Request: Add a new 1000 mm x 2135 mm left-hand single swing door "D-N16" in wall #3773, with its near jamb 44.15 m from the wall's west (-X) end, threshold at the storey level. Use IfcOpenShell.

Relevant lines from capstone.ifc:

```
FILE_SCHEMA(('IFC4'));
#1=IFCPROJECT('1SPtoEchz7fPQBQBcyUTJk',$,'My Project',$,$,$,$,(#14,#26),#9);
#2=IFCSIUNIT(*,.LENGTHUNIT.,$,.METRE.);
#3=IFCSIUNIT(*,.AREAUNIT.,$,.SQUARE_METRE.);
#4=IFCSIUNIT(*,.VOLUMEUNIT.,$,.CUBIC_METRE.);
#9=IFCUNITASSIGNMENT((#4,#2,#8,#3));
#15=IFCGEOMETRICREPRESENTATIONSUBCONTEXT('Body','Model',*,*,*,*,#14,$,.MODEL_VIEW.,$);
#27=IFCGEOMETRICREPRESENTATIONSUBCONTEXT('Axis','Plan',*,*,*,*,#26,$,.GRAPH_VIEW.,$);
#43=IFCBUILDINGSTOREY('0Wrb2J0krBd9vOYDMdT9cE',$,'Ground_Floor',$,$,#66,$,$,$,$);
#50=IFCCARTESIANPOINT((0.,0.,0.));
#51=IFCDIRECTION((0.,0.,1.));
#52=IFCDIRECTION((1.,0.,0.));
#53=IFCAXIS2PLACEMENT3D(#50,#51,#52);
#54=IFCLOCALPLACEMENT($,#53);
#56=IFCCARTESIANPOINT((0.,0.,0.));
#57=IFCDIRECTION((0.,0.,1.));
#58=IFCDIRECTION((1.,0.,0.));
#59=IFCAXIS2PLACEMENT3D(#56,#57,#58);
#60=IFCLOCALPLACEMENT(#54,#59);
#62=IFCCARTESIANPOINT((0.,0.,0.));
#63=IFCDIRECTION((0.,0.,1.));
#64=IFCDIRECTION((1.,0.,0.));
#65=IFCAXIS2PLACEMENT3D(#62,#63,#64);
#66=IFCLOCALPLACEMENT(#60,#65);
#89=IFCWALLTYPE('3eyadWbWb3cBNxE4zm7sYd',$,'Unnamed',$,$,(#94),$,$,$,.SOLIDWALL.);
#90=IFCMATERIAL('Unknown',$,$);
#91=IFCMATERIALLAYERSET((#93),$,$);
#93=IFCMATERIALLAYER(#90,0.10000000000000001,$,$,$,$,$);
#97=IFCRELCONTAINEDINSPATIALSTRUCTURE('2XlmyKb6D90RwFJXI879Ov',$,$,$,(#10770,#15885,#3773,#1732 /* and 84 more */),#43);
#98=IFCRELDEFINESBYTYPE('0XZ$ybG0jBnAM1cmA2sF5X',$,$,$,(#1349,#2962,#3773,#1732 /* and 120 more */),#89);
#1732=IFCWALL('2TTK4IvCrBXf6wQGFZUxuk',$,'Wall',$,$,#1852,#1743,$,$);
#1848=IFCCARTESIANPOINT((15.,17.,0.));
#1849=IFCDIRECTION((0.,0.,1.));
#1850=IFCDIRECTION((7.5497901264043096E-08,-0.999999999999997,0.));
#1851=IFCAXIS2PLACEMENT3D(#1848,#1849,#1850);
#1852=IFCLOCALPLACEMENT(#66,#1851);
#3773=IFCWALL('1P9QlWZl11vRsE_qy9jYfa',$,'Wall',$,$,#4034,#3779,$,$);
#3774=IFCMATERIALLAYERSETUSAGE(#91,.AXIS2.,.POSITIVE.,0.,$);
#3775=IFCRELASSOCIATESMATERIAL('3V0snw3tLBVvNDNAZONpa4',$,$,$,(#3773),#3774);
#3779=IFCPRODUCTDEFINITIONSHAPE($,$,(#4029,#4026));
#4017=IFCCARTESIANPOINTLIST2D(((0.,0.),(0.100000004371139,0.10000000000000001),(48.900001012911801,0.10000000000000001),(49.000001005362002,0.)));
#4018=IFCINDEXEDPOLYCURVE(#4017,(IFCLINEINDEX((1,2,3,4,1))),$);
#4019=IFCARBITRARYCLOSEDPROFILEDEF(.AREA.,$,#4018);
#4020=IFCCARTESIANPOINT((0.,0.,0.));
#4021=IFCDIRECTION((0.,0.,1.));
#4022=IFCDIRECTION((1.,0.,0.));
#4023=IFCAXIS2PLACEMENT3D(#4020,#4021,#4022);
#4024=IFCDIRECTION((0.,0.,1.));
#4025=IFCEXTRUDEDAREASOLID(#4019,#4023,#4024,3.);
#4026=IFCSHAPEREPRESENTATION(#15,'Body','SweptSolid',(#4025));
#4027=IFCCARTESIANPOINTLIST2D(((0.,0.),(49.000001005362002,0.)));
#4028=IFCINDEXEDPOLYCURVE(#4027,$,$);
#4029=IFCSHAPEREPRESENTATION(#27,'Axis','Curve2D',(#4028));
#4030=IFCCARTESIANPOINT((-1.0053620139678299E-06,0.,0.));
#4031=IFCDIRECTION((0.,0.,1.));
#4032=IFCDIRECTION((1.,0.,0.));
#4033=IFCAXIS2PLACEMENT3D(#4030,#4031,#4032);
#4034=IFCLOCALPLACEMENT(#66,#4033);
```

```python
import numpy as np
import ifcopenshell
import ifcopenshell.api.feature
import ifcopenshell.api.geometry
import ifcopenshell.api.root
import ifcopenshell.api.spatial
import ifcopenshell.geom
import ifcopenshell.util.element
import ifcopenshell.util.placement
import ifcopenshell.util.representation
import ifcopenshell.util.shape
import ifcopenshell.util.unit

model = ifcopenshell.open("capstone.ifc")
unit_scale = ifcopenshell.util.unit.calculate_unit_scale(model)
settings = ifcopenshell.geom.settings()


def volume(element):
    """Net volume in cubic metres, openings subtracted."""
    shape = ifcopenshell.geom.create_shape(settings, element)
    return ifcopenshell.util.shape.get_volume(shape.geometry)


wall = model.by_guid("1P9QlWZl11vRsE_qy9jYfa")
storey = ifcopenshell.util.element.get_container(wall, ifc_class="IfcBuildingStorey")
context = ifcopenshell.util.representation.get_context(model, "Model", "Body", "MODEL_VIEW")
before = volume(wall)

width, height, from_end, sill = 1, 2.135, 44.15, 0.0  # metres

# The wall runs along its own X axis, and the end named is its -X end.
wall_shape = ifcopenshell.geom.create_shape(settings, wall)
x, y, z = ifcopenshell.util.shape.get_vertices(wall_shape.geometry).T
start = x.min() + from_end
face, thickness = float(y.min()), float(y.max() - y.min())
wall_matrix = ifcopenshell.util.placement.get_local_placement(wall.ObjectPlacement)
level = ifcopenshell.util.placement.get_local_placement(storey.ObjectPlacement)[2, 3]


def in_wall(x, y):
    """Placement at x, y metres in the wall's axes, at sill height."""
    matrix = wall_matrix.copy()
    matrix[:, 3] = wall_matrix @ np.array([x / unit_scale, y / unit_scale, 0.0, 1.0])
    matrix[2, 3] = level + sill / unit_scale
    return matrix


# Opening: a box that overshoots both wall faces by 50 mm.
opening = ifcopenshell.api.root.create_entity(model, ifc_class="IfcOpeningElement", predefined_type="OPENING")
box = ifcopenshell.api.geometry.add_wall_representation(
    model, context=context, length=width, height=height, thickness=thickness + 0.1
)
ifcopenshell.api.geometry.assign_representation(model, product=opening, representation=box)
ifcopenshell.api.geometry.edit_object_placement(model, product=opening, matrix=in_wall(start, face - 0.05), is_si=False)
ifcopenshell.api.feature.add_feature(model, feature=opening, element=wall)

door = ifcopenshell.api.root.create_entity(model, ifc_class="IfcDoor", name="D-N16", predefined_type="DOOR")
door.OverallWidth, door.OverallHeight = width / unit_scale, height / unit_scale
door.OperationType = "SINGLE_SWING_LEFT"
body = ifcopenshell.api.geometry.add_door_representation(
    model,
    context=context,
    overall_width=door.OverallWidth,
    overall_height=door.OverallHeight,
    operation_type="SINGLE_SWING_LEFT",
    lining_properties={"LiningDepth": thickness / unit_scale, "ThresholdDepth": thickness / unit_scale},
)
ifcopenshell.api.geometry.assign_representation(model, product=door, representation=body)
ifcopenshell.api.spatial.assign_container(model, products=[door], relating_structure=storey)
ifcopenshell.api.feature.add_filling(model, opening=opening, element=door)

# The lining spans the wall, so the door starts at the wall face.
ifcopenshell.api.geometry.edit_object_placement(model, product=door, matrix=in_wall(start, face), is_si=False)

after = volume(wall)

print(f"wall volume {before:.3f} -> {after:.3f} m3")

model.write("capstone_rev.ifc")
```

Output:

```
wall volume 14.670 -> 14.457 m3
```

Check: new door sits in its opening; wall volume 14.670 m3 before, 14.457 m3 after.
